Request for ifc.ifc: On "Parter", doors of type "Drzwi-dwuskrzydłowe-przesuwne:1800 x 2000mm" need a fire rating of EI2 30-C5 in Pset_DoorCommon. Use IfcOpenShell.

First a look at what the model holds.

```python
import ifcopenshell
import ifcopenshell.util.element

model = ifcopenshell.open("ifc.ifc")
print(model.schema)
storey = next(s for s in model.by_type("IfcBuildingStorey") if s.Name == "Parter")
doors = [e for e in ifcopenshell.util.element.get_decomposition(storey) if e.is_a("IfcDoor")]
seen = {}
for e in doors:
    element_type = ifcopenshell.util.element.get_type(e)
    key = (element_type.Name if element_type != e and element_type else None, ifcopenshell.util.element.get_pset(e, "Pset_DoorCommon", "FireRating"))
    seen[key] = seen.get(key, 0) + 1
for (name, value), count in sorted(seen.items(), key=str):
    print(count, "x", name, "|", value)
```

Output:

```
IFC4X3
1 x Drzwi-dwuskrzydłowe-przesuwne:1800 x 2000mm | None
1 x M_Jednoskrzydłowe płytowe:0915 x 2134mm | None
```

```python
import ifcopenshell
import ifcopenshell.api.pset
import ifcopenshell.util.element

model = ifcopenshell.open("ifc.ifc")

storey = next(s for s in model.by_type("IfcBuildingStorey") if s.Name == "Parter")
doors = [e for e in ifcopenshell.util.element.get_decomposition(storey) if e.is_a("IfcDoor")]

count = 0
for e in doors:
    element_type = ifcopenshell.util.element.get_type(e)
    if element_type in (None, e) or element_type.Name != "Drzwi-dwuskrzydłowe-przesuwne:1800 x 2000mm":
        continue
    # add_pset returns the element's existing set when there is one.
    pset = ifcopenshell.api.pset.add_pset(model, product=e, name="Pset_DoorCommon")
    ifcopenshell.api.pset.edit_pset(model, pset=pset, properties={"FireRating": "EI2 30-C5"})
    count += 1

print(count, "doors updated")

model.write("ifc_updated.ifc")
```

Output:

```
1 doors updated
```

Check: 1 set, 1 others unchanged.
